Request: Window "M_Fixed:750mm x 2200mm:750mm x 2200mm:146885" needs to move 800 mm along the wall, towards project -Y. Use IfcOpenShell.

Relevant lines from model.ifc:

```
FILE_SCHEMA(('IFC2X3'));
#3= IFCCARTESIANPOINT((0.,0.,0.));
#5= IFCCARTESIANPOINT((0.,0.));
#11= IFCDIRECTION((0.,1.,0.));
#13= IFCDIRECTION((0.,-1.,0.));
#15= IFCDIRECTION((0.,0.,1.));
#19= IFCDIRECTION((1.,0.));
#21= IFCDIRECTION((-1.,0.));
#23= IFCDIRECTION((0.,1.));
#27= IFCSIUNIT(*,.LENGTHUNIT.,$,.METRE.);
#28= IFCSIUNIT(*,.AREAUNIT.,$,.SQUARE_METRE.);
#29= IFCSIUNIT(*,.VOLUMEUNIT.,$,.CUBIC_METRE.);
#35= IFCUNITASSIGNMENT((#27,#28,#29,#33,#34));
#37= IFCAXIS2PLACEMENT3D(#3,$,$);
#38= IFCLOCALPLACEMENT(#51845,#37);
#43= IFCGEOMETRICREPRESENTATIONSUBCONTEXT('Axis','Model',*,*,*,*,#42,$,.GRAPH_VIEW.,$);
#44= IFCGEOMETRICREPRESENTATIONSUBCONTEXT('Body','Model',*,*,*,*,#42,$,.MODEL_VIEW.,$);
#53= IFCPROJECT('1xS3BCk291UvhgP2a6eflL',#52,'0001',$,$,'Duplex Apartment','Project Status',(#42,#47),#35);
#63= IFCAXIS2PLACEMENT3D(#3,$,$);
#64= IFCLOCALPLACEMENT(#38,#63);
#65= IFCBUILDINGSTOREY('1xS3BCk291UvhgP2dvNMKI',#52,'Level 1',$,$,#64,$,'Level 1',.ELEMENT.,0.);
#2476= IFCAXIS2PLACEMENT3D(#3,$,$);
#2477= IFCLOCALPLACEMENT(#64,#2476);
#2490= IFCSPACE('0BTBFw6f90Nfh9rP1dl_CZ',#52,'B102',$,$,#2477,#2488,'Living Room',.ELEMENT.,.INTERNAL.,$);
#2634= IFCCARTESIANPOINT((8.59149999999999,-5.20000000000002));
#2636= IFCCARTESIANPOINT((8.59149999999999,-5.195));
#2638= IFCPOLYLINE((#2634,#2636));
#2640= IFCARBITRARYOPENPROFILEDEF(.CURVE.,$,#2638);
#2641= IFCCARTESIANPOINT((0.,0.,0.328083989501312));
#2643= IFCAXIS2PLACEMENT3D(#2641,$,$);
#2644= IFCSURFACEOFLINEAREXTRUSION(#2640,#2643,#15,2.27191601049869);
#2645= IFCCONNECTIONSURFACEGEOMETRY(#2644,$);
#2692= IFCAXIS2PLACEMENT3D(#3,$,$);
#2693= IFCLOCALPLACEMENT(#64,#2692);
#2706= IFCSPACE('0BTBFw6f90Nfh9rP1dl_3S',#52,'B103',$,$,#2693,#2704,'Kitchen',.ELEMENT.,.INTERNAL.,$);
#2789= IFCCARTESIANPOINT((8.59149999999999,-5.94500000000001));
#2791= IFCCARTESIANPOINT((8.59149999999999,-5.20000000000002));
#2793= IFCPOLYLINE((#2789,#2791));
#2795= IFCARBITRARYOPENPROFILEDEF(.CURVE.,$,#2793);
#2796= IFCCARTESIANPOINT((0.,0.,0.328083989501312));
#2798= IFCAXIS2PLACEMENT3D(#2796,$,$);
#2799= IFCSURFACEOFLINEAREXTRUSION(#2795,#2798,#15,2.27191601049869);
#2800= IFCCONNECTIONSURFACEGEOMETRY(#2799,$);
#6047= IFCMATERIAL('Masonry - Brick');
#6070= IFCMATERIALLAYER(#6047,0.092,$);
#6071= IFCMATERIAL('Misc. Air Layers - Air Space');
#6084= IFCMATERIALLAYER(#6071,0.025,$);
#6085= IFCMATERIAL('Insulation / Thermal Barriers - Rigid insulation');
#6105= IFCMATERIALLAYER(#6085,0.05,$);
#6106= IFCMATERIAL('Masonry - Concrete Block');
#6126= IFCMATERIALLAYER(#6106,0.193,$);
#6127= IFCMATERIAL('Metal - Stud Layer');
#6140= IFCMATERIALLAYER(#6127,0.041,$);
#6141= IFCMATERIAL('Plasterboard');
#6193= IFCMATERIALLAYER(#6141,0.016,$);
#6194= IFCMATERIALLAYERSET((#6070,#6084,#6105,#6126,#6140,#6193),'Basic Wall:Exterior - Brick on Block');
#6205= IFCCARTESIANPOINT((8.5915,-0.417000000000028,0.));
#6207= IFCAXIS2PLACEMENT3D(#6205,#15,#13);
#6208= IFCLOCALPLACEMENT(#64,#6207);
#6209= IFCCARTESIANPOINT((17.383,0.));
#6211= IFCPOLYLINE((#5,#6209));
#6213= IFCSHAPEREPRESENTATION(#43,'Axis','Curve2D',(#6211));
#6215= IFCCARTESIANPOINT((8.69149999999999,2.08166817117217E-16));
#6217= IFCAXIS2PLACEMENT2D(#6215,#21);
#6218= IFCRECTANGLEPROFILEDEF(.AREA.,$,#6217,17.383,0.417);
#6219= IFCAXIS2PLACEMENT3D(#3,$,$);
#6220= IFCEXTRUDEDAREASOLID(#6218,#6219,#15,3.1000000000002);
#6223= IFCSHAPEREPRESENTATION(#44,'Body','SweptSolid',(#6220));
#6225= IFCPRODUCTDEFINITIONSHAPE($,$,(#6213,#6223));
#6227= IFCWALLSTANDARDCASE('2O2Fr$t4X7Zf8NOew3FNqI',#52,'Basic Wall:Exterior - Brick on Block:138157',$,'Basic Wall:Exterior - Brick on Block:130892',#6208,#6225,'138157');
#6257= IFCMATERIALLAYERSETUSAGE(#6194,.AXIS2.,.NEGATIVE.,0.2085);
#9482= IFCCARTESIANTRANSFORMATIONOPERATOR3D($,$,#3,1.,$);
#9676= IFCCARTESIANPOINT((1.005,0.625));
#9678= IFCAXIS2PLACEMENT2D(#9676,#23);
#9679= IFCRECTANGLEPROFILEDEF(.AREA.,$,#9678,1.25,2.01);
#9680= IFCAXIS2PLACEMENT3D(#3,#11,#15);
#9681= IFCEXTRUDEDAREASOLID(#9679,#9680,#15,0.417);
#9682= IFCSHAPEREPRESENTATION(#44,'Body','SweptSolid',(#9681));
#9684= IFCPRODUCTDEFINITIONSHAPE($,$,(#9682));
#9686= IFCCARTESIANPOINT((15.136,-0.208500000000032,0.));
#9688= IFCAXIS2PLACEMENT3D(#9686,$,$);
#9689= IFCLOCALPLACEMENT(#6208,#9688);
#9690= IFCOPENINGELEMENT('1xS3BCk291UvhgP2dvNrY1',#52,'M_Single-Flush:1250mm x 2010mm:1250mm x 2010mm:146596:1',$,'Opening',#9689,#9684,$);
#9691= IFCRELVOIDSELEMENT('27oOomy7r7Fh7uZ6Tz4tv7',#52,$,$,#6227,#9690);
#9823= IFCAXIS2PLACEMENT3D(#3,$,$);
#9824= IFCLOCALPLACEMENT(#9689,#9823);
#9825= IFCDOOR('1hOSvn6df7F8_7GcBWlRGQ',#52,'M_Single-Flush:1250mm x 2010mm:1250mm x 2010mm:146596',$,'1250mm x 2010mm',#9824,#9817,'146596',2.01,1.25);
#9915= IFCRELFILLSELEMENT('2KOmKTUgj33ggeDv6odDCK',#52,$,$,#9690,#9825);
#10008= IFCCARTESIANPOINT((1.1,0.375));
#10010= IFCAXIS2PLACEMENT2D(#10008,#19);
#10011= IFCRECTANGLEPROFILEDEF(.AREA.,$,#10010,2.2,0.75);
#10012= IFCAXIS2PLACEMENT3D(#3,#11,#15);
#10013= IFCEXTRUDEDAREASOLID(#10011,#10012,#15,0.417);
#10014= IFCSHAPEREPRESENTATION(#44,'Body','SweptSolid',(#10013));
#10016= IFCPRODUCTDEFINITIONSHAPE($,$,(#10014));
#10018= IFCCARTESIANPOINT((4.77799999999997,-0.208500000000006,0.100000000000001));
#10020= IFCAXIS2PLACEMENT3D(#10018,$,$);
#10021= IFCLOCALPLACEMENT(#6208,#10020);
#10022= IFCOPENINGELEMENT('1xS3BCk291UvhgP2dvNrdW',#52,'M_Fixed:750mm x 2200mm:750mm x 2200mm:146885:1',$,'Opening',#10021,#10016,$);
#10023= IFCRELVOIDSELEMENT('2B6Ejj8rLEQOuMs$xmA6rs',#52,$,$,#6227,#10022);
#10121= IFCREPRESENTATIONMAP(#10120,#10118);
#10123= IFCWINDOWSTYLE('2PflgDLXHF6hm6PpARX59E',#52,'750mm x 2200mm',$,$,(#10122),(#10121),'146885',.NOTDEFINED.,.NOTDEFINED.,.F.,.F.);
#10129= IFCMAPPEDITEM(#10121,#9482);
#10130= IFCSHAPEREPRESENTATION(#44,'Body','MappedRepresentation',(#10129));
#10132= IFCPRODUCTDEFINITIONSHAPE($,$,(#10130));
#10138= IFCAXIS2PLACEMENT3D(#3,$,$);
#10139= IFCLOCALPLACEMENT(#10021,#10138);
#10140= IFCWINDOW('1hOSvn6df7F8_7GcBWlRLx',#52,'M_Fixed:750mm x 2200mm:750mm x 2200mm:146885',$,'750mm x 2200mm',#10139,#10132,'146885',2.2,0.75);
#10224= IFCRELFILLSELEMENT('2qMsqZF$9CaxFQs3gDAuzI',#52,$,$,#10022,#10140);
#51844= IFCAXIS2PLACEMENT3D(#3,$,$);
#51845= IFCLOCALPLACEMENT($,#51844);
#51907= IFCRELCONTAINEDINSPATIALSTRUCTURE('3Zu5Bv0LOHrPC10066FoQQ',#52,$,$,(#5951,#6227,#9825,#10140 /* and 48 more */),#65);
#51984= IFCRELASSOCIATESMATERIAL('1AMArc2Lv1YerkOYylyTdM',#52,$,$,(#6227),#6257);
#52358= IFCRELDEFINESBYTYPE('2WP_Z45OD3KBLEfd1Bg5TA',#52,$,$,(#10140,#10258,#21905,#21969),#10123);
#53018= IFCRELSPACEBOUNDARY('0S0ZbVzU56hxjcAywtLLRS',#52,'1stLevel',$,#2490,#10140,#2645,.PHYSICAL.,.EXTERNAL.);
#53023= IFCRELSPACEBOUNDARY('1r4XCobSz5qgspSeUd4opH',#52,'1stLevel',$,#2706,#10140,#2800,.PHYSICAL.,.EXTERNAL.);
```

```python
import numpy as np
import ifcopenshell
import ifcopenshell.api.geometry
import ifcopenshell.util.placement
import ifcopenshell.util.unit

model = ifcopenshell.open("model.ifc")
unit_scale = ifcopenshell.util.unit.calculate_unit_scale(model)

window = model.by_id(10140)
opening = window.FillsVoids[0].RelatingOpeningElement
wall = opening.VoidsElements[0].RelatingBuildingElement

wall_matrix = ifcopenshell.util.placement.get_local_placement(wall.ObjectPlacement)
shift = wall_matrix[:3, 0] * 0.8 / unit_scale
before = ifcopenshell.util.placement.get_local_placement(window.ObjectPlacement)[:3, 3].copy()

# The window is placed relative to its opening, so it follows when the opening moves.
matrix = ifcopenshell.util.placement.get_local_placement(opening.ObjectPlacement)
matrix[:3, 3] += shift
ifcopenshell.api.geometry.edit_object_placement(
    model, product=opening, matrix=matrix, is_si=False, should_transform_children=True
)

# Space boundary surfaces are stored in each space's coordinates; move them too.
for rel in window.ProvidesBoundaries:
    if not rel.ConnectionGeometry:
        continue
    surface = rel.ConnectionGeometry.SurfaceOnRelatingElement
    space_matrix = ifcopenshell.util.placement.get_local_placement(rel.RelatingSpace.ObjectPlacement)
    point = np.array(surface.Position.Location.Coordinates) + space_matrix[:3, :3].T @ shift
    surface.Position = model.createIfcAxis2Placement3D(
        model.createIfcCartesianPoint(point.tolist()), surface.Position.Axis, surface.Position.RefDirection
    )

after = ifcopenshell.util.placement.get_local_placement(window.ObjectPlacement)[:3, 3]
print("window moved by", (after - before).round(3) + 0.0)

model.write("model_updated.ifc")
```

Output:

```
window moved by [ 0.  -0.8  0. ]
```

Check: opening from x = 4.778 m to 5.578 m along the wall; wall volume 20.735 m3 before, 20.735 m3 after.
